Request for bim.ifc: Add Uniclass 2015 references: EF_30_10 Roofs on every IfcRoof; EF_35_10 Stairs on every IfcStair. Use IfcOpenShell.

First a look at what the model holds.

```python
import ifcopenshell

model = ifcopenshell.open("bim.ifc")
print(model.schema)
print("classifications:", [c.Name for c in model.by_type("IfcClassification")])
for ifc_class in ("IfcDoor", "IfcRoof", "IfcStair", "IfcWall", "IfcWindow"):
    print(ifc_class, len(model.by_type(ifc_class)))
```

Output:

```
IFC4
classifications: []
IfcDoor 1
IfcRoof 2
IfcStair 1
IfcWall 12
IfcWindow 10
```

```python
import ifcopenshell
import ifcopenshell.api.classification

model = ifcopenshell.open("bim.ifc")

system = ifcopenshell.api.classification.add_classification(model, classification="Uniclass 2015")

codes = {
    "IfcRoof": ("EF_30_10", "Roofs"),
    "IfcStair": ("EF_35_10", "Stairs"),
}
for ifc_class, (code, name) in codes.items():
    products = model.by_type(ifc_class)
    ifcopenshell.api.classification.add_reference(
        model, products=products, classification=system, identification=code, name=name
    )
    print(code, len(products))

model.write("bim_edited.ifc")
```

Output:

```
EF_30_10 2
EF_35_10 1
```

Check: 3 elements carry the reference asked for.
